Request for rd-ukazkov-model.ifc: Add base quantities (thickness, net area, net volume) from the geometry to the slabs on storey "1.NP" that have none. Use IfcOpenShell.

First a look at what the model holds.

```python
import ifcopenshell
import ifcopenshell.util.element
import ifcopenshell.util.unit

model = ifcopenshell.open("rd-ukazkov-model.ifc")
print(model.schema)
for unit_type in ("LENGTHUNIT", "AREAUNIT", "VOLUMEUNIT"):
    print(unit_type, ifcopenshell.util.unit.calculate_unit_scale(model, unit_type))
storey = next(s for s in model.by_type("IfcBuildingStorey") if s.Name == "1.NP")
slabs = [e for e in ifcopenshell.util.element.get_decomposition(storey) if e.is_a("IfcSlab")]
for e in sorted(slabs, key=lambda e: e.id()):
    print(e.id(), e.is_a(), e.Name, list(ifcopenshell.util.element.get_psets(e, qtos_only=True)), sep=" | ")
```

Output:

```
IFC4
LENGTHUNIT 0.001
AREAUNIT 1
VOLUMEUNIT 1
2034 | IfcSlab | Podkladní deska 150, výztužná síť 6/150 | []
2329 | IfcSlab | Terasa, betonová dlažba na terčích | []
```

```python
import ifcopenshell
import ifcopenshell.api.pset
import ifcopenshell.geom
import ifcopenshell.util.element
import ifcopenshell.util.shape
import ifcopenshell.util.unit

model = ifcopenshell.open("rd-ukazkov-model.ifc")
unit_scale = ifcopenshell.util.unit.calculate_unit_scale(model)
area_scale = ifcopenshell.util.unit.calculate_unit_scale(model, "AREAUNIT")
volume_scale = ifcopenshell.util.unit.calculate_unit_scale(model, "VOLUMEUNIT")
settings = ifcopenshell.geom.settings()

storey = next(s for s in model.by_type("IfcBuildingStorey") if s.Name == "1.NP")
slabs = [e for e in ifcopenshell.util.element.get_decomposition(storey) if e.is_a("IfcSlab")]

for e in sorted(slabs, key=lambda e: e.id()):
    if ifcopenshell.util.element.get_psets(e, qtos_only=True, should_inherit=False):
        continue
    # Geometry comes back in metres, in the element's own axes.
    shape = ifcopenshell.geom.create_shape(settings, e)
    values = {
        "Width": ifcopenshell.util.shape.get_z(shape.geometry) / unit_scale,
        "NetArea": ifcopenshell.util.shape.get_footprint_area(shape.geometry) / area_scale,
        "NetVolume": ifcopenshell.util.shape.get_volume(shape.geometry) / volume_scale,
    }
    qto = ifcopenshell.api.pset.add_qto(model, product=e, name="Qto_SlabBaseQuantities")
    ifcopenshell.api.pset.edit_qto(model, qto=qto, properties=values)
    print(e.id(), {k: round(v, 3) for k, v in values.items()})

model.write("rd-ukazkov-model_rev.ifc")
```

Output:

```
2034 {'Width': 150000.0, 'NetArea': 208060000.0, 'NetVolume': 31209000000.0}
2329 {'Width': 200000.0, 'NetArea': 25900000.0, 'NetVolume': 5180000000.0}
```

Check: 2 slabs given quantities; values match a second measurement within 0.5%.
